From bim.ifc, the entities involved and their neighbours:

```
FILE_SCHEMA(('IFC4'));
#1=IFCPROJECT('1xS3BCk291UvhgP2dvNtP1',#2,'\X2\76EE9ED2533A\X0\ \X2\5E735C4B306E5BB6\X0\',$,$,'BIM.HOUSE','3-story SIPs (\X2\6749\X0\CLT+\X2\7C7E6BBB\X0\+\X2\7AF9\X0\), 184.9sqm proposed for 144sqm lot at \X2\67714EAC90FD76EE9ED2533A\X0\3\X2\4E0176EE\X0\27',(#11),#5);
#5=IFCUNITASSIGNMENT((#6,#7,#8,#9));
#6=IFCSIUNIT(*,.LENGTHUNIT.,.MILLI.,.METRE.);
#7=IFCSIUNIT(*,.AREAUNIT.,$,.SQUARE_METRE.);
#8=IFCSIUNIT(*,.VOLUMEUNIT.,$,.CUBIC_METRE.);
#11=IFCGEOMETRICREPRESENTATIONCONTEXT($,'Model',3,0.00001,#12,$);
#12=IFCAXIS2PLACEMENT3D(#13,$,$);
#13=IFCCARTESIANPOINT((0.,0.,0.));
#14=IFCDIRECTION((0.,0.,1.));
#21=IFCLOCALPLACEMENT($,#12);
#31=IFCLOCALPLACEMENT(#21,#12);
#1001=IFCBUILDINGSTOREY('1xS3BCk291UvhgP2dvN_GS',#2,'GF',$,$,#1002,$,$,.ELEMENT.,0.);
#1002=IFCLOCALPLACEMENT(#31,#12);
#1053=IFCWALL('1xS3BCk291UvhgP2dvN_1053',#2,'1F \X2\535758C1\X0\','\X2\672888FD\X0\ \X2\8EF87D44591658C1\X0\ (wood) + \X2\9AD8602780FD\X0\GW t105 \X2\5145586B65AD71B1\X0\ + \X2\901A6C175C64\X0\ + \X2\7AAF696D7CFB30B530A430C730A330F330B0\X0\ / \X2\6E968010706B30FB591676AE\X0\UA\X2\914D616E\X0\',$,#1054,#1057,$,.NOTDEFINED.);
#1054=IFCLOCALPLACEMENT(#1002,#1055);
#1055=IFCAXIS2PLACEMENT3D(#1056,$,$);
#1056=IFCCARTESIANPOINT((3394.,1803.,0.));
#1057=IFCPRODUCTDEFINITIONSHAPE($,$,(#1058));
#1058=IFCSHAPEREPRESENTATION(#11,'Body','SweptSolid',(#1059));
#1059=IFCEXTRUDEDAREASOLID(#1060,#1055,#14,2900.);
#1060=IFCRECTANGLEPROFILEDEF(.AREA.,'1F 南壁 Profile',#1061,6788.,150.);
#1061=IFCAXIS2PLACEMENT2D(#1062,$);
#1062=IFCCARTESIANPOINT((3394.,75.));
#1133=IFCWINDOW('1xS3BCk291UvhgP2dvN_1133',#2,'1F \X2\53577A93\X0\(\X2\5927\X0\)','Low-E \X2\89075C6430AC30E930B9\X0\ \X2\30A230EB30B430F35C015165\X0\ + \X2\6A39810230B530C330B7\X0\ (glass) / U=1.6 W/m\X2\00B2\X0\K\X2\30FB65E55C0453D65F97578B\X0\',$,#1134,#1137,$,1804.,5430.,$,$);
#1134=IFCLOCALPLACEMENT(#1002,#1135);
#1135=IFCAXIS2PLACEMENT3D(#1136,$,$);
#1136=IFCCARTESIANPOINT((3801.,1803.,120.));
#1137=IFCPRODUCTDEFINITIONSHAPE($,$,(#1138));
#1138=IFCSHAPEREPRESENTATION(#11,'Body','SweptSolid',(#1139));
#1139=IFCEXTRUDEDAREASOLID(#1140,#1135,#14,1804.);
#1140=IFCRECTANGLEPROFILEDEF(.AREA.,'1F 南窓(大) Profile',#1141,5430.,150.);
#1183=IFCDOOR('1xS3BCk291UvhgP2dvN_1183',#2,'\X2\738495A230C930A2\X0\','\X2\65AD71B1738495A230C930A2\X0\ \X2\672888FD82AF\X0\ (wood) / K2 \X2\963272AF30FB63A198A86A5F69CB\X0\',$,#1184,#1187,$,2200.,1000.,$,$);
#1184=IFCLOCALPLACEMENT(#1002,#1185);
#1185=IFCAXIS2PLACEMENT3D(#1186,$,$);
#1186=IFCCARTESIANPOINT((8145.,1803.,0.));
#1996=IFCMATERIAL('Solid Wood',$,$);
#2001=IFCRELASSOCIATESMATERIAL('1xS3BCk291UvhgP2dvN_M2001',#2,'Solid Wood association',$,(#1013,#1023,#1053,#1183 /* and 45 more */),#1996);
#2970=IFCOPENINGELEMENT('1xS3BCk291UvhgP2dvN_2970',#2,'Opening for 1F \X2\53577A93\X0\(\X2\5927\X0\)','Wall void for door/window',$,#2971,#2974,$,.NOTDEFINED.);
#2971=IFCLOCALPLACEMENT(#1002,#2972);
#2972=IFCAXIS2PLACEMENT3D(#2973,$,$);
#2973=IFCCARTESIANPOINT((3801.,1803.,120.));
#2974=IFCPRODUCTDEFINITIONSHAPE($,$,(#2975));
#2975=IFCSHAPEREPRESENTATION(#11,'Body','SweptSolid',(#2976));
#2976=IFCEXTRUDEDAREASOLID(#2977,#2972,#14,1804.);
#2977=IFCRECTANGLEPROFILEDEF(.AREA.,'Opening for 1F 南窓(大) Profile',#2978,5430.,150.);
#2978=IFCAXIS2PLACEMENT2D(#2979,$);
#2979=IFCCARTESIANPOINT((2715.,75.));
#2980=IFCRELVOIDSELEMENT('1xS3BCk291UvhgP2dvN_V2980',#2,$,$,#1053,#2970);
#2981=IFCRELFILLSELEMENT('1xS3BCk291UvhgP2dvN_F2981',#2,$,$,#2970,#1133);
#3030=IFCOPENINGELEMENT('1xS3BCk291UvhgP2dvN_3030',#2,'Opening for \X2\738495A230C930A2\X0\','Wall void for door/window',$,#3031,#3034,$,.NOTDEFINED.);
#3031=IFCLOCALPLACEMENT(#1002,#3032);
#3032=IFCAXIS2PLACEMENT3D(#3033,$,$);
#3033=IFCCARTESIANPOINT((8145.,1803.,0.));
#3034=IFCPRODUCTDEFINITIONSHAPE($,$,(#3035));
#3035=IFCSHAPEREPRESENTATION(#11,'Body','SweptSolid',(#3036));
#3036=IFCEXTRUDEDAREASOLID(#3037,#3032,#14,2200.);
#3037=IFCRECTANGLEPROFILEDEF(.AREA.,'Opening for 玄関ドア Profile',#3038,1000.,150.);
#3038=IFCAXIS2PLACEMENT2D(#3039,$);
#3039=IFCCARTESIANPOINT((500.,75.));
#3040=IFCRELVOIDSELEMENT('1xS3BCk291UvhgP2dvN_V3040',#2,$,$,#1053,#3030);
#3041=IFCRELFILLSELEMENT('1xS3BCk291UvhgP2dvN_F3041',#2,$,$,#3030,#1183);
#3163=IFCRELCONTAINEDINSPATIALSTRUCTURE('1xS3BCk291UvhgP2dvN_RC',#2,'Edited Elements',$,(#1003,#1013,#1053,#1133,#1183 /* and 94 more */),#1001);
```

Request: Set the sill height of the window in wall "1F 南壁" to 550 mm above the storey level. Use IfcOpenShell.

```python
import numpy as np
import ifcopenshell
import ifcopenshell.api.geometry
import ifcopenshell.geom
import ifcopenshell.util.element
import ifcopenshell.util.placement
import ifcopenshell.util.shape
import ifcopenshell.util.unit

model = ifcopenshell.open("bim.ifc")
unit_scale = ifcopenshell.util.unit.calculate_unit_scale(model)

window = model.by_id(1133)
opening = window.FillsVoids[0].RelatingOpeningElement
storey = ifcopenshell.util.element.get_container(window, ifc_class="IfcBuildingStorey")
level = ifcopenshell.util.placement.get_local_placement(storey.ObjectPlacement)[2, 3]

# The opening's origin need not be at the sill, so measure its lowest point.
shape = ifcopenshell.geom.create_shape(ifcopenshell.geom.settings(), opening)
bottom = ifcopenshell.util.shape.get_shape_bottom_elevation(shape, shape.geometry) / unit_scale
dz = level + 550.0 - bottom

shift = np.array([0.0, 0.0, dz])
# The window is not placed relative to its opening, so move both.
for product in (opening, window):
    matrix = ifcopenshell.util.placement.get_local_placement(product.ObjectPlacement)
    matrix[:3, 3] += shift
    ifcopenshell.api.geometry.edit_object_placement(model, product=product, matrix=matrix, is_si=False)

print(f"moved by {dz * unit_scale:+.3f} m")

model.write("bim-out.ifc")
```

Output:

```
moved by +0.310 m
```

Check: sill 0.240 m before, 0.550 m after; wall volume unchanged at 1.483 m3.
